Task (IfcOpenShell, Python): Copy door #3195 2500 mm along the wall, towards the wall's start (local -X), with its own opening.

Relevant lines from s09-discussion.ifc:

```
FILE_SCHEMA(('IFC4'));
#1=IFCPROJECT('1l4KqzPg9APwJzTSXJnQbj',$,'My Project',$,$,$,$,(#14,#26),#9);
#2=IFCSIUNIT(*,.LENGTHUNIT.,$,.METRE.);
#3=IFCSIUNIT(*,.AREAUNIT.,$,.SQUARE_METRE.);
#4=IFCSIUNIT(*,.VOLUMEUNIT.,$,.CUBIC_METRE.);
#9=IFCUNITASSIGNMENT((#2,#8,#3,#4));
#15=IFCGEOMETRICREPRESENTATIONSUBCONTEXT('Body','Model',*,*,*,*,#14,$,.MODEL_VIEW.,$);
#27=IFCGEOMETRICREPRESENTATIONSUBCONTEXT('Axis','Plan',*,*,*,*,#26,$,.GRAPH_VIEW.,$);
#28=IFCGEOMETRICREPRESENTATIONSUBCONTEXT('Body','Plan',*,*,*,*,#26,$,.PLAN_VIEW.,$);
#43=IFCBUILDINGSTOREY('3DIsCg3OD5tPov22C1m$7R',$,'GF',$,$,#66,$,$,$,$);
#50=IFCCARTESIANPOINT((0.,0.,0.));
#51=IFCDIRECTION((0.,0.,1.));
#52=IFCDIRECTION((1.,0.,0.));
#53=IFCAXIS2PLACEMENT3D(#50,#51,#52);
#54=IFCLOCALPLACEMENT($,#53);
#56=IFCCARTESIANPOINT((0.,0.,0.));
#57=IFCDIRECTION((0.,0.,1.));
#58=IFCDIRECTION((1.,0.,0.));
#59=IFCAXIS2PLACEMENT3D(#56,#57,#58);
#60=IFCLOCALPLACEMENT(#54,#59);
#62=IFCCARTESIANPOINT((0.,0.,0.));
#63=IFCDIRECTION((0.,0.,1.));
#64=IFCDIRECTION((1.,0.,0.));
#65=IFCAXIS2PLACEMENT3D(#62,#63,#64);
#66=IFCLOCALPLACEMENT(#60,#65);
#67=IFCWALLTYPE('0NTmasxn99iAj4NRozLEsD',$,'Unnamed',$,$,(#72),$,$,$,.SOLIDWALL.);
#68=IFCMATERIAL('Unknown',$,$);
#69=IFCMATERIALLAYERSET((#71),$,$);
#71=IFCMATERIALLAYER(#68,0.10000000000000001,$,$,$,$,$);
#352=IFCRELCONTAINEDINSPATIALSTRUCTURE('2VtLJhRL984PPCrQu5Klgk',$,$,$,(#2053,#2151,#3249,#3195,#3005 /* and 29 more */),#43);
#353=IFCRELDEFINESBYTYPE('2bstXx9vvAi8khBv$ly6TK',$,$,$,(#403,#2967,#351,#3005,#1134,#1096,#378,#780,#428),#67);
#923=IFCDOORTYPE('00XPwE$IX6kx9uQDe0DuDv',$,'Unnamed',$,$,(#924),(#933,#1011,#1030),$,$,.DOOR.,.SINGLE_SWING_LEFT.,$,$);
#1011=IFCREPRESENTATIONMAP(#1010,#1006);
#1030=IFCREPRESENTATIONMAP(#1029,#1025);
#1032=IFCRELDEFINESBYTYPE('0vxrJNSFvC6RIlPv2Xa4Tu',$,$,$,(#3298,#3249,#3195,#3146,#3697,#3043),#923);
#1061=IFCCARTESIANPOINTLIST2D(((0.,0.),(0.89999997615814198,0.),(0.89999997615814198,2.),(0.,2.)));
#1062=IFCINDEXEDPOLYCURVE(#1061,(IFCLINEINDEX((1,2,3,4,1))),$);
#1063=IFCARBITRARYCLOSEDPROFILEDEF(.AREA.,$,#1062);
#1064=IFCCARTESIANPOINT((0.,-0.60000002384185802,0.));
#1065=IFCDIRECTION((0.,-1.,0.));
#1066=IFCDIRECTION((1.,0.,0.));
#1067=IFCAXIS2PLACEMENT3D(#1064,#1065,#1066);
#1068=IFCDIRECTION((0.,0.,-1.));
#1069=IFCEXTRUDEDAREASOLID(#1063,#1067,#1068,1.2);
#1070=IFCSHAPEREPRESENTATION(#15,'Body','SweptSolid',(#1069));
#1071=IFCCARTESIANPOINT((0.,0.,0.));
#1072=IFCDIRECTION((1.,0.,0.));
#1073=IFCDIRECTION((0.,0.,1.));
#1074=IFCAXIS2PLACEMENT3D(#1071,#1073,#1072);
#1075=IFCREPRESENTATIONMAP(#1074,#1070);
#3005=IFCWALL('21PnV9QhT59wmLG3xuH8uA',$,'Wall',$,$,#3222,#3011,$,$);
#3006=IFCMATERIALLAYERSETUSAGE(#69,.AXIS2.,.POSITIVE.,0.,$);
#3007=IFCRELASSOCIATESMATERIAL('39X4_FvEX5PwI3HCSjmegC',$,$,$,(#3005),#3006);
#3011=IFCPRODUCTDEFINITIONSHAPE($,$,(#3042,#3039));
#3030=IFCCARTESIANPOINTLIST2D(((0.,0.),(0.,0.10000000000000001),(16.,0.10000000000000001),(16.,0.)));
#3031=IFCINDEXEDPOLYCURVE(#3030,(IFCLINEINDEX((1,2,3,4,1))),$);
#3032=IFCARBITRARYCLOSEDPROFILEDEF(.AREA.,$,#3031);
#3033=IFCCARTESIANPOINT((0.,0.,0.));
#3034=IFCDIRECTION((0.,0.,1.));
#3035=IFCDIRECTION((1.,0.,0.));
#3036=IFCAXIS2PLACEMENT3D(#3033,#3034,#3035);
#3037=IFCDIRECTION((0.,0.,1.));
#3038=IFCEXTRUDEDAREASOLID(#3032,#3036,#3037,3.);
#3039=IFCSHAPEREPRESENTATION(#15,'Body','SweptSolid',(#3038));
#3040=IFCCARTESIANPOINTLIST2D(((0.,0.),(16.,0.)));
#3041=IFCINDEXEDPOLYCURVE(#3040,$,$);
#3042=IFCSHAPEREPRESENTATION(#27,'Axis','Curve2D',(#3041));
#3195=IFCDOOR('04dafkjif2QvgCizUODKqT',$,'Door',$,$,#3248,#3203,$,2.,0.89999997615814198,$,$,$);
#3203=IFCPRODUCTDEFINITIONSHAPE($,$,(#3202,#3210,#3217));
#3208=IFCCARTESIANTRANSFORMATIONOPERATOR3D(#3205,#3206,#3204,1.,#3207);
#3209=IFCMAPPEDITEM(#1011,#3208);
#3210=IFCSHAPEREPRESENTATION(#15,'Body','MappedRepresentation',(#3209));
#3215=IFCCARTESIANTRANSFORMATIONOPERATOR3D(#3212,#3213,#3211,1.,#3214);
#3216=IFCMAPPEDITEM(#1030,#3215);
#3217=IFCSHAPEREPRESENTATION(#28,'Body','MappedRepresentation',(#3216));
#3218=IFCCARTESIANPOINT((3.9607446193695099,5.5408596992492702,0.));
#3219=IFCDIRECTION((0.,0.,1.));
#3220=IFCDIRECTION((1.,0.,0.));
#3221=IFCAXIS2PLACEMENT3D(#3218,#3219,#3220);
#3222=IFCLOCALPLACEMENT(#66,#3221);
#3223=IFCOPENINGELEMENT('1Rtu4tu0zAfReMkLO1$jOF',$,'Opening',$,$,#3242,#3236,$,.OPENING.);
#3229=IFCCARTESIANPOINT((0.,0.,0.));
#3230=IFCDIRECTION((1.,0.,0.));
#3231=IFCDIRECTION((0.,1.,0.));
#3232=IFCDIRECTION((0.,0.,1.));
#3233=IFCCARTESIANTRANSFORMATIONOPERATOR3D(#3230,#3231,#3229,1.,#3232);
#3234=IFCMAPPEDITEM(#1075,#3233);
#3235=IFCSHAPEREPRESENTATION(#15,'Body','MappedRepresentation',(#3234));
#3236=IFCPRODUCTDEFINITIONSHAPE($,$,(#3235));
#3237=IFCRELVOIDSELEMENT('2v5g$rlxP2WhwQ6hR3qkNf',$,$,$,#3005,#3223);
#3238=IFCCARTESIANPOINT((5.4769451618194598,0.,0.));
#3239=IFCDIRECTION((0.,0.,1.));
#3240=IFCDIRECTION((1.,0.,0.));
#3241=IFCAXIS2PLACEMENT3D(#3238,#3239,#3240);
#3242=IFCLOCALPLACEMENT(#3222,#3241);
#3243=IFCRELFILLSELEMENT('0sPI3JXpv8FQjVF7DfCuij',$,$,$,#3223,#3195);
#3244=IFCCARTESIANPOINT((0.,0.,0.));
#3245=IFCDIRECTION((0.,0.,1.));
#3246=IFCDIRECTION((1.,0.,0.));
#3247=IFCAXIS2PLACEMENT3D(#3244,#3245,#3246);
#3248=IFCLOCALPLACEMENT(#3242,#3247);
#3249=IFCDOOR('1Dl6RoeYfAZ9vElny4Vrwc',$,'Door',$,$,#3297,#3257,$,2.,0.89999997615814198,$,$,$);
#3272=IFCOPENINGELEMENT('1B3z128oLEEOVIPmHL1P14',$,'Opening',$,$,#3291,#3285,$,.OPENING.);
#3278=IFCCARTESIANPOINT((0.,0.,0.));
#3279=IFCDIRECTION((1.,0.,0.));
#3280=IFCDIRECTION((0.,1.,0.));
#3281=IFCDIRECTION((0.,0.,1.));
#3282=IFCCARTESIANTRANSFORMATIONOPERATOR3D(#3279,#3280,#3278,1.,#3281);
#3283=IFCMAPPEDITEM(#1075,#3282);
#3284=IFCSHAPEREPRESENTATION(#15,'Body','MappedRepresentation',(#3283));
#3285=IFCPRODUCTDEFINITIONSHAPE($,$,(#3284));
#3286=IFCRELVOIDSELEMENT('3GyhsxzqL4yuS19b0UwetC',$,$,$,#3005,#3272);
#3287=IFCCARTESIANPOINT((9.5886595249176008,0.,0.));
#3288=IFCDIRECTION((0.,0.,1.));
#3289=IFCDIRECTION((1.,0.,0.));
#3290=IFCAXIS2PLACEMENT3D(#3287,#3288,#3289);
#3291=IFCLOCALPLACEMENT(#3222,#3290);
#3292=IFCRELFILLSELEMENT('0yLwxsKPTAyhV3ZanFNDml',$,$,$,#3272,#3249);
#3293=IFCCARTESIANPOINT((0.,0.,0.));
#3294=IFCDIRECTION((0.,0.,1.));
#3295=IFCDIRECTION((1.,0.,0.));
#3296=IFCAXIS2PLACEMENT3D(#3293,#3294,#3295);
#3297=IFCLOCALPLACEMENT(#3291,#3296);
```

```python
import ifcopenshell
import ifcopenshell.api.feature
import ifcopenshell.api.geometry
import ifcopenshell.api.root
import ifcopenshell.geom
import ifcopenshell.util.element
import ifcopenshell.util.placement
import ifcopenshell.util.shape
import ifcopenshell.util.unit

model = ifcopenshell.open("s09-discussion.ifc")
unit_scale = ifcopenshell.util.unit.calculate_unit_scale(model)
settings = ifcopenshell.geom.settings()


def volume(element):
    """Net volume in cubic metres, openings subtracted."""
    shape = ifcopenshell.geom.create_shape(settings, element)
    return ifcopenshell.util.shape.get_volume(shape.geometry)


door = model.by_guid("04dafkjif2QvgCizUODKqT")
opening = door.FillsVoids[0].RelatingOpeningElement
wall = opening.VoidsElements[0].RelatingBuildingElement
before = volume(wall)
shift = ifcopenshell.util.placement.get_local_placement(wall.ObjectPlacement)[:3, 0] * -2.5 / unit_scale

# copy_class copies the void relationship, type, container and properties, but no geometry.
new_opening = ifcopenshell.api.root.copy_class(model, product=opening)
new_opening.Representation = ifcopenshell.util.element.copy_deep(
    model, opening.Representation, exclude=["IfcGeometricRepresentationContext", "IfcRepresentationMap"]
)
new_door = ifcopenshell.api.root.copy_class(model, product=door)
new_door.Representation = ifcopenshell.util.element.copy_deep(
    model, door.Representation, exclude=["IfcGeometricRepresentationContext", "IfcRepresentationMap"]
)
ifcopenshell.api.feature.add_filling(model, opening=new_opening, element=new_door)

for old, new in ((opening, new_opening), (door, new_door)):
    matrix = ifcopenshell.util.placement.get_local_placement(old.ObjectPlacement)
    matrix[:3, 3] += shift
    ifcopenshell.api.geometry.edit_object_placement(model, product=new, matrix=matrix, is_si=False)

after = volume(wall)

print(f"wall volume {before:.3f} -> {after:.3f} m3")

model.write("s09-discussion_edited.ifc")
```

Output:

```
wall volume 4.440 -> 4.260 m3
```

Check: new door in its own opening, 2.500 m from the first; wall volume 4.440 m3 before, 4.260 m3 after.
